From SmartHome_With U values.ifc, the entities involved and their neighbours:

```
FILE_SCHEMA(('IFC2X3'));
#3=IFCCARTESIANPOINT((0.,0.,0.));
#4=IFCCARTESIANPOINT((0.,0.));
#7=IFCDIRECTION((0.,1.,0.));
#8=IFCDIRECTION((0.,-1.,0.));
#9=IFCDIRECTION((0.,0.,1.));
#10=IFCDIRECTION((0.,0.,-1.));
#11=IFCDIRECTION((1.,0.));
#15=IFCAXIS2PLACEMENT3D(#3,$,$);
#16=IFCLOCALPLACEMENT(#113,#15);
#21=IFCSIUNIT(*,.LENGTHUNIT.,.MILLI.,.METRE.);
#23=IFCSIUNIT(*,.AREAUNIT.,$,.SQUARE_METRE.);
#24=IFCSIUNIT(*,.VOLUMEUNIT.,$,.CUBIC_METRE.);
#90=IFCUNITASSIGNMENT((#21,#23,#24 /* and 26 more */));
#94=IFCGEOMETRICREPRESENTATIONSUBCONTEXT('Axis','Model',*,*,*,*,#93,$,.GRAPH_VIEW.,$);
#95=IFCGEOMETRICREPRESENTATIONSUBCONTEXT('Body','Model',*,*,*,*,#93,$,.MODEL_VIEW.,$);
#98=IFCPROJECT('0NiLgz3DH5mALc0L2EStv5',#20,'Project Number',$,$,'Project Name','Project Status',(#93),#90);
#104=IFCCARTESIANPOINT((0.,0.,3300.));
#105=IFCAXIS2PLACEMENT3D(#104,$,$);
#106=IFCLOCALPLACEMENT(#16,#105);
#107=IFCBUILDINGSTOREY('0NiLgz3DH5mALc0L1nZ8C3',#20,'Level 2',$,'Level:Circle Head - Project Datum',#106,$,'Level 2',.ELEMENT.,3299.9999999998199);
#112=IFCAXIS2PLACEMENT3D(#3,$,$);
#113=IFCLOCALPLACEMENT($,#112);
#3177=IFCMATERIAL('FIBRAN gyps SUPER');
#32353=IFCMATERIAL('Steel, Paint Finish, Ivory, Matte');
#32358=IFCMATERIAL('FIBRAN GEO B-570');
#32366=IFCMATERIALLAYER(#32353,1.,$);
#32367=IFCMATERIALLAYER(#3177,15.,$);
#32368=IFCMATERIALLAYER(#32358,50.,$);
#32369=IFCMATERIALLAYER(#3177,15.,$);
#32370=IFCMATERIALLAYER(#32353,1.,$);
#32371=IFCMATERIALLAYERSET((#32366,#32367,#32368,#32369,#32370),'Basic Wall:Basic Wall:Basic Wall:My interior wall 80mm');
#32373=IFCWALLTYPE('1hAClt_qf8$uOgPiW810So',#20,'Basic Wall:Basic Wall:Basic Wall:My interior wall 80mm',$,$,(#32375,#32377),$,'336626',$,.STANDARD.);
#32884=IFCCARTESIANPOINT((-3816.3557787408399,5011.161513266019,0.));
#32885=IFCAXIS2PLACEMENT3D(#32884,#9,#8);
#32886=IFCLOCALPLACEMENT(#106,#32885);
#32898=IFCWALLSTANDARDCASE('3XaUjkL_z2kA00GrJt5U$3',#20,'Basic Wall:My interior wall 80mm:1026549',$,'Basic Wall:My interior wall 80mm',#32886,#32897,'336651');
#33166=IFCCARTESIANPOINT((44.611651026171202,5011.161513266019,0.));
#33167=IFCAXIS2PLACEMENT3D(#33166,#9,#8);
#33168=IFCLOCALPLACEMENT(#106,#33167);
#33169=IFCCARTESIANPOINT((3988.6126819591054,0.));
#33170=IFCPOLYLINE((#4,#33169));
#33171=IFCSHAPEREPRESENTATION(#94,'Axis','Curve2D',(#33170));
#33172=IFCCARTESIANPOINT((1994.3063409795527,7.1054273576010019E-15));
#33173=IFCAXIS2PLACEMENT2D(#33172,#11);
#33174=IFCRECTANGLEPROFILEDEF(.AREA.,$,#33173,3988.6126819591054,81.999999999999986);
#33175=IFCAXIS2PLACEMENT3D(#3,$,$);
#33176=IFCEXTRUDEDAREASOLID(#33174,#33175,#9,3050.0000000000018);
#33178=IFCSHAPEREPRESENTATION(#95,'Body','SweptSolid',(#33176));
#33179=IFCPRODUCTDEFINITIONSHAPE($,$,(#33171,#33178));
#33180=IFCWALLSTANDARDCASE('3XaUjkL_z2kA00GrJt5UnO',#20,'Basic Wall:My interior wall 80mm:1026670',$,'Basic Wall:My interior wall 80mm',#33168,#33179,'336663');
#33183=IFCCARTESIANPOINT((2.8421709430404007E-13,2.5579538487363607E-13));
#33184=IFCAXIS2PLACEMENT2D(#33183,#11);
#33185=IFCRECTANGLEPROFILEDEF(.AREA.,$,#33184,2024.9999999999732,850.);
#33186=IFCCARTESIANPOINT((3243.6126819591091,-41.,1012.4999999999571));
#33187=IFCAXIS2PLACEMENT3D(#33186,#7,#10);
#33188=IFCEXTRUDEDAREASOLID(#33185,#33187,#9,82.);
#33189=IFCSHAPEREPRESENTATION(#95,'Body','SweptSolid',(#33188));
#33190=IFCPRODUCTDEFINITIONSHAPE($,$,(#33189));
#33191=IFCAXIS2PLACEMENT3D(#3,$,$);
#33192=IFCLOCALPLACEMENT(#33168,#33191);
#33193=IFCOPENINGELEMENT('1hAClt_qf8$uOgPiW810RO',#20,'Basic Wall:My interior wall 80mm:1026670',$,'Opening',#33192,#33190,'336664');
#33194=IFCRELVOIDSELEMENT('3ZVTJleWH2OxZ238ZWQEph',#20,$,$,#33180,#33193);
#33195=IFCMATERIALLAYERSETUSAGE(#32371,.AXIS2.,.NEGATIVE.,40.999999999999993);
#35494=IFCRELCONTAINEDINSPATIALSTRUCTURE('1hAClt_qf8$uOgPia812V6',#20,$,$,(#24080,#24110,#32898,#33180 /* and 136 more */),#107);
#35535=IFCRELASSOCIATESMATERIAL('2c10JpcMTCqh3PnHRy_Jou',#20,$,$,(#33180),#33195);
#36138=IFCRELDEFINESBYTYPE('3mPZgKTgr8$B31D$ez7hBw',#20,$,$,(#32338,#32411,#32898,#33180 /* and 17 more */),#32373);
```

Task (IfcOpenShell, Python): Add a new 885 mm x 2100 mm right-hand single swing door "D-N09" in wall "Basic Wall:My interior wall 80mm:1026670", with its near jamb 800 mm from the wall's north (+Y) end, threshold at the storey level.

```python
import numpy as np
import ifcopenshell
import ifcopenshell.api.feature
import ifcopenshell.api.geometry
import ifcopenshell.api.root
import ifcopenshell.api.spatial
import ifcopenshell.api.type
import ifcopenshell.geom
import ifcopenshell.util.element
import ifcopenshell.util.placement
import ifcopenshell.util.representation
import ifcopenshell.util.shape
import ifcopenshell.util.unit

model = ifcopenshell.open("SmartHome_With U values.ifc")
unit_scale = ifcopenshell.util.unit.calculate_unit_scale(model)
settings = ifcopenshell.geom.settings()


def volume(element):
    """Net volume in cubic metres, openings subtracted."""
    shape = ifcopenshell.geom.create_shape(settings, element)
    return ifcopenshell.util.shape.get_volume(shape.geometry)


wall = model.by_guid("3XaUjkL_z2kA00GrJt5UnO")
storey = ifcopenshell.util.element.get_container(wall, ifc_class="IfcBuildingStorey")
context = ifcopenshell.util.representation.get_context(model, "Model", "Body", "MODEL_VIEW")
before = volume(wall)

width, height, from_end, sill = 0.885, 2.1, 0.8, 0.0  # metres

# The wall runs along its own X axis, and the end named is its -X end.
wall_shape = ifcopenshell.geom.create_shape(settings, wall)
x, y, z = ifcopenshell.util.shape.get_vertices(wall_shape.geometry).T
start = x.min() + from_end
face, thickness = float(y.min()), float(y.max() - y.min())
wall_matrix = ifcopenshell.util.placement.get_local_placement(wall.ObjectPlacement)
level = ifcopenshell.util.placement.get_local_placement(storey.ObjectPlacement)[2, 3]


def in_wall(x, y):
    """Placement at x, y metres in the wall's axes, at sill height."""
    matrix = wall_matrix.copy()
    matrix[:, 3] = wall_matrix @ np.array([x / unit_scale, y / unit_scale, 0.0, 1.0])
    matrix[2, 3] = level + sill / unit_scale
    return matrix


# Opening: a box that overshoots both wall faces by 50 mm.
opening = ifcopenshell.api.root.create_entity(model, ifc_class="IfcOpeningElement")
box = ifcopenshell.api.geometry.add_wall_representation(
    model, context=context, length=width, height=height, thickness=thickness + 0.1
)
ifcopenshell.api.geometry.assign_representation(model, product=opening, representation=box)
ifcopenshell.api.geometry.edit_object_placement(model, product=opening, matrix=in_wall(start, face - 0.05), is_si=False)
ifcopenshell.api.feature.add_feature(model, feature=opening, element=wall)

door = ifcopenshell.api.root.create_entity(model, ifc_class="IfcDoor", name="D-N09")
door.OverallWidth, door.OverallHeight = width / unit_scale, height / unit_scale
body = ifcopenshell.api.geometry.add_door_representation(
    model,
    context=context,
    overall_width=door.OverallWidth,
    overall_height=door.OverallHeight,
    operation_type="SINGLE_SWING_RIGHT",
    lining_properties={"LiningDepth": thickness / unit_scale, "ThresholdDepth": thickness / unit_scale},
)
ifcopenshell.api.geometry.assign_representation(model, product=door, representation=body)
ifcopenshell.api.spatial.assign_container(model, products=[door], relating_structure=storey)
fills = ifcopenshell.api.feature.add_filling(model, opening=opening, element=door)
fills.OwnerHistory = door.OwnerHistory  # required in IFC2X3

# IFC2X3 keeps the operation on the door style.
style = ifcopenshell.api.root.create_entity(model, ifc_class="IfcDoorStyle", name="D-N09")
style.OperationType, style.ConstructionType = "SINGLE_SWING_RIGHT", "NOTDEFINED"
style.ParameterTakesPrecedence = style.Sizeable = False
ifcopenshell.api.type.assign_type(model, related_objects=[door], relating_type=style)

# The lining spans the wall, so the door starts at the wall face.
ifcopenshell.api.geometry.edit_object_placement(model, product=door, matrix=in_wall(start, face), is_si=False)

after = volume(wall)

print(f"wall volume {before:.3f} -> {after:.3f} m3")

model.write("SmartHome_With U values-out.ifc")
```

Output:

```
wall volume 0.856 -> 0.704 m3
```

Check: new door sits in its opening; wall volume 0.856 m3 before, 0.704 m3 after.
